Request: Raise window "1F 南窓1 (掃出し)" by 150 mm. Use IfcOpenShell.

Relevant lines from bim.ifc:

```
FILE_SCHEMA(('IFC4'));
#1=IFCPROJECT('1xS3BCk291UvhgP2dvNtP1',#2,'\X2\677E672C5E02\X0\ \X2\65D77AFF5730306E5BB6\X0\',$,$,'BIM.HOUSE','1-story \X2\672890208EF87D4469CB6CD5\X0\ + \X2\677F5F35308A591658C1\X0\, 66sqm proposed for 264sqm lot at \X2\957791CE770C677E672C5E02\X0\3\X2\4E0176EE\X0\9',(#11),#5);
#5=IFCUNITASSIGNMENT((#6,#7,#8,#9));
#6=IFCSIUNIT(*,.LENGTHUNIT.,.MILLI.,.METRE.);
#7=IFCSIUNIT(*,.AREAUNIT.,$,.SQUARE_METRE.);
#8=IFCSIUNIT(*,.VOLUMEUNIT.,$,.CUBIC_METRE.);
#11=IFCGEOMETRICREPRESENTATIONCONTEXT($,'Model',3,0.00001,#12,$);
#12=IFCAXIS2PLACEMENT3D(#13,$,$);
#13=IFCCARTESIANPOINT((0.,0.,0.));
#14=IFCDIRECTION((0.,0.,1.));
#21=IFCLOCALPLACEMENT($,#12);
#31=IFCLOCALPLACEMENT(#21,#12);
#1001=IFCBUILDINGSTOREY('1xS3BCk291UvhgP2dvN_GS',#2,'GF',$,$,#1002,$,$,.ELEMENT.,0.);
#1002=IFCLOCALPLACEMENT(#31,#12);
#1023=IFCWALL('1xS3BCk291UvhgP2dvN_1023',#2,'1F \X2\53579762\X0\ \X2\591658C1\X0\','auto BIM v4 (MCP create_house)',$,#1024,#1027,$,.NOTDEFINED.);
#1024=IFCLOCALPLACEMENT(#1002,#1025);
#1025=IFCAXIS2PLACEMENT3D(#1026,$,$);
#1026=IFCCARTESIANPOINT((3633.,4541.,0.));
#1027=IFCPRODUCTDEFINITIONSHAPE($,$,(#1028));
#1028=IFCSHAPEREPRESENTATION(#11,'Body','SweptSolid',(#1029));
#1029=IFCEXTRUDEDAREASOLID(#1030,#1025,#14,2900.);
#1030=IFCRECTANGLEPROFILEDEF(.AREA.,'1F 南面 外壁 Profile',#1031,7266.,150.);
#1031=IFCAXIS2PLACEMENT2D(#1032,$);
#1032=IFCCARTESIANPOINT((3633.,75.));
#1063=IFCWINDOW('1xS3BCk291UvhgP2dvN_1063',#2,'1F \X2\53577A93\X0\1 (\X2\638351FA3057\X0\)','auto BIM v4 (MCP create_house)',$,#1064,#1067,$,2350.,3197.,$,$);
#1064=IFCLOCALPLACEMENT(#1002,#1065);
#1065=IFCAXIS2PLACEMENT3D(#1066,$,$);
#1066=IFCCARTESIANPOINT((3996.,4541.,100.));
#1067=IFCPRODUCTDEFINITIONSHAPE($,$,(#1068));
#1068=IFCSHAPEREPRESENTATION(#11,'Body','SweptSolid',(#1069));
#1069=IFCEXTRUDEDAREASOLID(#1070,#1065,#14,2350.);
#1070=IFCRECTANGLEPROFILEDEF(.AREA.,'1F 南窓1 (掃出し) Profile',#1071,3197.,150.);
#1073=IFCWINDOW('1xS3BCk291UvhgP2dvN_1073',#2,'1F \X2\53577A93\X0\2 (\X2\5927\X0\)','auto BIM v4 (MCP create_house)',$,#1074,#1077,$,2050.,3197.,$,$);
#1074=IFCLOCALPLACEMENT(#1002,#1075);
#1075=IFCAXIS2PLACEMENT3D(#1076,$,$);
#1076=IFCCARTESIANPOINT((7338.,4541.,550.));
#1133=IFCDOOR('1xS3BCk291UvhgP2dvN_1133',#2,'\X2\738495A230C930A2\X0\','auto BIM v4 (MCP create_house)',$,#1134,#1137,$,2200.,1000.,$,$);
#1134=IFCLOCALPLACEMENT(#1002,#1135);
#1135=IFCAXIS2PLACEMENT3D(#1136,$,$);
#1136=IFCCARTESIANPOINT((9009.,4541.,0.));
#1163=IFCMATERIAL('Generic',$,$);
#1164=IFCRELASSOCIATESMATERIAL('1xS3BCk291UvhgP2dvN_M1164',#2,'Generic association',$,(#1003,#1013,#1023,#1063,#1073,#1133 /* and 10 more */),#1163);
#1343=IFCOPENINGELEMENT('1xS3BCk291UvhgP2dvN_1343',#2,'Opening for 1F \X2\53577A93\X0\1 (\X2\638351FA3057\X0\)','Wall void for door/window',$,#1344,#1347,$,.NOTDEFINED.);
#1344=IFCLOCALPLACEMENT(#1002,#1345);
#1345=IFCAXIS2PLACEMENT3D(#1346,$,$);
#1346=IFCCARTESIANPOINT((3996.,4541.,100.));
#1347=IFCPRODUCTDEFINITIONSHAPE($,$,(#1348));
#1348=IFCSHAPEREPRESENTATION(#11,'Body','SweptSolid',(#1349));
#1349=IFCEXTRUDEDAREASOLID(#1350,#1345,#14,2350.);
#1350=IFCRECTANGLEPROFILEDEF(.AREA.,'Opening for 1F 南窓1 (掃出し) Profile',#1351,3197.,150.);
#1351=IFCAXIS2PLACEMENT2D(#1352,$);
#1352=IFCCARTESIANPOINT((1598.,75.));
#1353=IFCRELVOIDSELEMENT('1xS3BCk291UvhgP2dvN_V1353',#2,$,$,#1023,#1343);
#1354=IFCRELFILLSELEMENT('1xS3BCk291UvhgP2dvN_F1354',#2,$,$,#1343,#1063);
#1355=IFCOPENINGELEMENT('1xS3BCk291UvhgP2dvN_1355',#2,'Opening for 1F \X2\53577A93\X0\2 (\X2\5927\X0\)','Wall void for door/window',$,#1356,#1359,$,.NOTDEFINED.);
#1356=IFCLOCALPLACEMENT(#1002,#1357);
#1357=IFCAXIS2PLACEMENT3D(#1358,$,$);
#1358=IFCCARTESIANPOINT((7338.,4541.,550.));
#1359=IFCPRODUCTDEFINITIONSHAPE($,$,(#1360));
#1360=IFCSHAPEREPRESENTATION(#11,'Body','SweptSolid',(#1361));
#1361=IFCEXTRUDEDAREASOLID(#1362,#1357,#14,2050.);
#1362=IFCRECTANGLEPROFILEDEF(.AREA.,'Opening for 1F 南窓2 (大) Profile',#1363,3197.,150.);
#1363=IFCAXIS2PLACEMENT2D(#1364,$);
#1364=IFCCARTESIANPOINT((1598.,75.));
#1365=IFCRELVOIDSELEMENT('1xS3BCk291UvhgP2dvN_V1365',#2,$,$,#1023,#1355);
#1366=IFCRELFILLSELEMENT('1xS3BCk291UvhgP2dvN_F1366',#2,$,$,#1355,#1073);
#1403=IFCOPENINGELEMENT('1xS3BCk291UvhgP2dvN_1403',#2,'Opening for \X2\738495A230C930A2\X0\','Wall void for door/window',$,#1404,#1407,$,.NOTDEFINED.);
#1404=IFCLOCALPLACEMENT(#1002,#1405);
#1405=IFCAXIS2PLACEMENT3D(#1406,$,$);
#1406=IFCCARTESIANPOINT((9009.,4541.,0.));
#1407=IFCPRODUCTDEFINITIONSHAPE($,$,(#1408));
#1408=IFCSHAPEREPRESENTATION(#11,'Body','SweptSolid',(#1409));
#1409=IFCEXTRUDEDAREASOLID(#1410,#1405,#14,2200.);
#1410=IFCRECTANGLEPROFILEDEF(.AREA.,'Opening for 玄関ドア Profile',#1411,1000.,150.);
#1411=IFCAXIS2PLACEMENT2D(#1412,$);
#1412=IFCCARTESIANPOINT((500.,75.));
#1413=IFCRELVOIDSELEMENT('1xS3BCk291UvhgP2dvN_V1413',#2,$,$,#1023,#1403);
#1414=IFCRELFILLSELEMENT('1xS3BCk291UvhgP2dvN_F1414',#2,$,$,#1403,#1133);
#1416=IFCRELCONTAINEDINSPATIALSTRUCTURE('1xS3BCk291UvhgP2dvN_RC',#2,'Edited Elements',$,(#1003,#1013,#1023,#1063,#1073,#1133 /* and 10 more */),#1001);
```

```python
import numpy as np
import ifcopenshell
import ifcopenshell.api.geometry
import ifcopenshell.util.placement
import ifcopenshell.util.unit

model = ifcopenshell.open("bim.ifc")
unit_scale = ifcopenshell.util.unit.calculate_unit_scale(model)

window = model.by_guid("1xS3BCk291UvhgP2dvN_1063")
opening = window.FillsVoids[0].RelatingOpeningElement
dz = 0.15 / unit_scale

shift = np.array([0.0, 0.0, dz])
# The window is not placed relative to its opening, so move both.
for product in (opening, window):
    matrix = ifcopenshell.util.placement.get_local_placement(product.ObjectPlacement)
    matrix[:3, 3] += shift
    ifcopenshell.api.geometry.edit_object_placement(model, product=product, matrix=matrix, is_si=False)

print(f"moved by {dz * unit_scale:+.3f} m")

model.write("bim-out.ifc")
```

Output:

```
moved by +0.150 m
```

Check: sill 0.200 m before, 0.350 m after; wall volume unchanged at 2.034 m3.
